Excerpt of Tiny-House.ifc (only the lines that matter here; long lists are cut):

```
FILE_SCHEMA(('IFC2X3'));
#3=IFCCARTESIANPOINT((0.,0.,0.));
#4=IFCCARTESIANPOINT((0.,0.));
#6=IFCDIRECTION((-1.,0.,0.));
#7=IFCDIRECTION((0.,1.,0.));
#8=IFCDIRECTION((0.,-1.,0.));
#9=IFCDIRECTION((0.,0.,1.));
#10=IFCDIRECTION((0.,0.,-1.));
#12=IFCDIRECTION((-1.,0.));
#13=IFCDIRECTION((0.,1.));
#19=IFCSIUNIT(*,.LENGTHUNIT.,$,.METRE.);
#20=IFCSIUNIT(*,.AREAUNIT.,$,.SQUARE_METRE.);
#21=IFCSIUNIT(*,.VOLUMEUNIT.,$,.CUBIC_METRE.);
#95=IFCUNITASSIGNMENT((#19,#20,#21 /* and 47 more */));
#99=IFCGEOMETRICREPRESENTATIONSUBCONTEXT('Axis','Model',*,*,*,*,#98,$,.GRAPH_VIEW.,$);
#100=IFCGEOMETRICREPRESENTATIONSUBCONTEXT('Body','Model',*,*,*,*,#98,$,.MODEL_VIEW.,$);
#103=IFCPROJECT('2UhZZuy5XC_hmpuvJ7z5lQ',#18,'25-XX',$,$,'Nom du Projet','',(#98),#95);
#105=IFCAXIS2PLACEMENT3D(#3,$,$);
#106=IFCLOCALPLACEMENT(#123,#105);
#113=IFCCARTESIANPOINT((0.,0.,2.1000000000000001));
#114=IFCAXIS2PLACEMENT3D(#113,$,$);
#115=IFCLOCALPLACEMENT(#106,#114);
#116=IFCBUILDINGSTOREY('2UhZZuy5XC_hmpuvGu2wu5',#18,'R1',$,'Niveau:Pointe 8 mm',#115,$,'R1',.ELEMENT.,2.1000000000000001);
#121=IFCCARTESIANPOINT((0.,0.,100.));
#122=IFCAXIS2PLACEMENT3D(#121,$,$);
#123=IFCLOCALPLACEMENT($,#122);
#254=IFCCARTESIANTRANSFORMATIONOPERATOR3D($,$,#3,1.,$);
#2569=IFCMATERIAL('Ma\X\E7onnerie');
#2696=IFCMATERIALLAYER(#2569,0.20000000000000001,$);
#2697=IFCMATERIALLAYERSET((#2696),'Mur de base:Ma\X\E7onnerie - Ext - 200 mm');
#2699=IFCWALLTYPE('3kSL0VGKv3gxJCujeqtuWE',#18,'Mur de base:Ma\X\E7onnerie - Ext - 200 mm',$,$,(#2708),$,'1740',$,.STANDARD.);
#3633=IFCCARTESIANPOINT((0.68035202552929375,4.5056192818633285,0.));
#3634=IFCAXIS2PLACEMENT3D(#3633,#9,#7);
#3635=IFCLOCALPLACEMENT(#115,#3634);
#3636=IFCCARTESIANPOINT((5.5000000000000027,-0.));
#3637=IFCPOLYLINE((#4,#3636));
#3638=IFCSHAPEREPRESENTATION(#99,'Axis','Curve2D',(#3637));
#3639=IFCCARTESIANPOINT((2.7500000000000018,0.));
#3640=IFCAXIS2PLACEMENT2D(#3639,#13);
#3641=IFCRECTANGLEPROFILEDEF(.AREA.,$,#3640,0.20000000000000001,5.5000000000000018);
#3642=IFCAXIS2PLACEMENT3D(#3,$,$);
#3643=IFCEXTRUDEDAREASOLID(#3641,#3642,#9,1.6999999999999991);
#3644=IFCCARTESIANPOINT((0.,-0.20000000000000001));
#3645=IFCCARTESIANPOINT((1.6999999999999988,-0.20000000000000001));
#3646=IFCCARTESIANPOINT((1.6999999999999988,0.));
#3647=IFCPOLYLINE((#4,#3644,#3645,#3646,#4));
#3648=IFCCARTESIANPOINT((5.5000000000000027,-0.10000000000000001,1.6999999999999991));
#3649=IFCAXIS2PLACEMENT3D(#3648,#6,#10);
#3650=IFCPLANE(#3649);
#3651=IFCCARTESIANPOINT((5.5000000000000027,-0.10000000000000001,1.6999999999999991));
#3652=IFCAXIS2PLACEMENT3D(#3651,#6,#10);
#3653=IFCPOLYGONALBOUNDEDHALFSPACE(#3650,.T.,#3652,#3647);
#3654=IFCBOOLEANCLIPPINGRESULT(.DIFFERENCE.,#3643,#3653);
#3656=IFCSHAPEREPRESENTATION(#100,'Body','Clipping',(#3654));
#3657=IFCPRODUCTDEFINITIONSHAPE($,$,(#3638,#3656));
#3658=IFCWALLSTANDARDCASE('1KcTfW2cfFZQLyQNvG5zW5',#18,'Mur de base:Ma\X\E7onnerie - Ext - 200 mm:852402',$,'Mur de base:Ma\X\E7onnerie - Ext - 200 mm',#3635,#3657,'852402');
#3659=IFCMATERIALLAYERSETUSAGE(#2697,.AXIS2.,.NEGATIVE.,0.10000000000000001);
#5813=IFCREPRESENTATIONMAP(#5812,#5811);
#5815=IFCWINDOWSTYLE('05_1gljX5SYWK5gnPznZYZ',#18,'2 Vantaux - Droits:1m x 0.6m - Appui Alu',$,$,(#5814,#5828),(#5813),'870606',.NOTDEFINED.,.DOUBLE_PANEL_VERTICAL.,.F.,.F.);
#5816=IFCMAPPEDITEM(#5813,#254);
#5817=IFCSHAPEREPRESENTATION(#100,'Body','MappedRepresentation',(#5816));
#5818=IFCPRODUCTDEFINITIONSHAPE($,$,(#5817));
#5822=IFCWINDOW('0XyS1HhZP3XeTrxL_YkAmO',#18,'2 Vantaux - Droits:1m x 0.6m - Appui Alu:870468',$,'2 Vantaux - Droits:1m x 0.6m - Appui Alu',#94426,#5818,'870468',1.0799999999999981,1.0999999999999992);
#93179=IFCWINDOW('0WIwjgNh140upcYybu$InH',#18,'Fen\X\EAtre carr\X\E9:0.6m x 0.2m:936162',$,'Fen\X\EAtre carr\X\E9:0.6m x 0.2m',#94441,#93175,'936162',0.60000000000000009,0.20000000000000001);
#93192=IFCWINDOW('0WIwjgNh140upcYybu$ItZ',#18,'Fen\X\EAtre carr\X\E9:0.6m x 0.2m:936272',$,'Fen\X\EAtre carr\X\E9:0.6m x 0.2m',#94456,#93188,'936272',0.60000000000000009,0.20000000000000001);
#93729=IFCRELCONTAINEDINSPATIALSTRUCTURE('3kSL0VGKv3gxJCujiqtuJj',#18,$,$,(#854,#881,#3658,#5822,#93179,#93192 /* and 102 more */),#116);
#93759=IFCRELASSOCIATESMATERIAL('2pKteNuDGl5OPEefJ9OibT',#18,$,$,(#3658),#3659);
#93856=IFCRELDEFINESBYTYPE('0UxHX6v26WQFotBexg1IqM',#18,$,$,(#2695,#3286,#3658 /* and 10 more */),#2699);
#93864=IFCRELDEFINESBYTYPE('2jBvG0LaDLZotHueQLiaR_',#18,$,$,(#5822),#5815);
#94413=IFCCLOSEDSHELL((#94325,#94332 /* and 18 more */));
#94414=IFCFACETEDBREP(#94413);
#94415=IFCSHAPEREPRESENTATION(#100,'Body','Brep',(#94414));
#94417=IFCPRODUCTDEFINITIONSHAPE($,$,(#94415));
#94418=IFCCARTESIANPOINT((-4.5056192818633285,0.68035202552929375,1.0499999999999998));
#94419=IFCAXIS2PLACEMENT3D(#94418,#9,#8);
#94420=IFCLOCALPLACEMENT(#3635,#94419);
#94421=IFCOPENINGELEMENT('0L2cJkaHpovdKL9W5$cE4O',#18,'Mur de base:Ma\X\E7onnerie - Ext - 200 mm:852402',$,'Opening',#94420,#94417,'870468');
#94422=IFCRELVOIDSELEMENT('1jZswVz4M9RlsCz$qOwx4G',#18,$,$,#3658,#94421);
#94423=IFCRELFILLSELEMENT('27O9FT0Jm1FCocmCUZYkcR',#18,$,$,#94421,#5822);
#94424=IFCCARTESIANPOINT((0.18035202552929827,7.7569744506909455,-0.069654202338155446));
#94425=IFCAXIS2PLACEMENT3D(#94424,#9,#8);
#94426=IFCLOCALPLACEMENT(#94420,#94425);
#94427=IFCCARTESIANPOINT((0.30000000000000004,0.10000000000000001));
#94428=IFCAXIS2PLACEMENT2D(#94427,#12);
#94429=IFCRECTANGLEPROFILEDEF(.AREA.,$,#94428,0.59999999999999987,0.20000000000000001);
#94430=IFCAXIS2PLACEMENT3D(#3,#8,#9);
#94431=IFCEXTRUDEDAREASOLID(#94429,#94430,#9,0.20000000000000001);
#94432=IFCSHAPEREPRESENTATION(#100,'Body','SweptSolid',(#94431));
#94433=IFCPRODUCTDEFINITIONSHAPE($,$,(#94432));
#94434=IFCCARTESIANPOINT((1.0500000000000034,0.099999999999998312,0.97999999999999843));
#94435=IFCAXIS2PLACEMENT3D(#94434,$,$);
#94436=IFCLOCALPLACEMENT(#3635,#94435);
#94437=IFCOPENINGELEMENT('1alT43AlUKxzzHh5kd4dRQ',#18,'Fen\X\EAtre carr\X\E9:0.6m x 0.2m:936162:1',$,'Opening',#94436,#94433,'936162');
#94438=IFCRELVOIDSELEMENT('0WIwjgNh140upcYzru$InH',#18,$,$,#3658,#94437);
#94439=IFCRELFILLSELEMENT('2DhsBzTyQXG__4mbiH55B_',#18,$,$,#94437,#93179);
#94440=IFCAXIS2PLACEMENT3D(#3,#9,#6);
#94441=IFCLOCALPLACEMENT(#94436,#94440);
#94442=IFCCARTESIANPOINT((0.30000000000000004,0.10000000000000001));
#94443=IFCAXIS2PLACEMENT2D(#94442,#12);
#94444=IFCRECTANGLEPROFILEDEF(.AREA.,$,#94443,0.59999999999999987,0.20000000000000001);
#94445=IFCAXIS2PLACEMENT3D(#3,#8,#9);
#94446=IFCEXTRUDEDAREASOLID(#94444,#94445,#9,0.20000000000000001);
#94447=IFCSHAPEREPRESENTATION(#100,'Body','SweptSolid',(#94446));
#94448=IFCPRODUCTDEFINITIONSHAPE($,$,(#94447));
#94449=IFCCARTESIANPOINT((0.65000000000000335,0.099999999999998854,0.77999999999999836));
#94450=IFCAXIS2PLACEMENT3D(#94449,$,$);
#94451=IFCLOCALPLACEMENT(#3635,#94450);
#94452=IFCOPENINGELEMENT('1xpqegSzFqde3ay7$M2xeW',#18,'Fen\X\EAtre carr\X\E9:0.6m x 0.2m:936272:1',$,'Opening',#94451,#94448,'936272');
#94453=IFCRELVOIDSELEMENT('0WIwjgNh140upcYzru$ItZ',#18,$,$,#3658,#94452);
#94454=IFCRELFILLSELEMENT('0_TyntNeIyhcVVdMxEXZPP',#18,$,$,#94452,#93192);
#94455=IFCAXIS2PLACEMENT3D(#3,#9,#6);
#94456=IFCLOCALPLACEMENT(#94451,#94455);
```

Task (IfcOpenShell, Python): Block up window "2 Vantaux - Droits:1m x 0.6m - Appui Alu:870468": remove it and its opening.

```python
import ifcopenshell
import ifcopenshell.api.feature
import ifcopenshell.api.root
import ifcopenshell.geom
import ifcopenshell.util.shape

model = ifcopenshell.open("Tiny-House.ifc")
settings = ifcopenshell.geom.settings()


def volume(element):
    """Net volume in cubic metres, openings subtracted."""
    shape = ifcopenshell.geom.create_shape(settings, element)
    return ifcopenshell.util.shape.get_volume(shape.geometry)


window = model.by_guid("0XyS1HhZP3XeTrxL_YkAmO")
opening = window.FillsVoids[0].RelatingOpeningElement
wall = opening.VoidsElements[0].RelatingBuildingElement
before = volume(wall)

ifcopenshell.api.root.remove_product(model, product=window)
ifcopenshell.api.feature.remove_feature(model, feature=opening)

after = volume(wall)

print(f"wall volume {before:.3f} -> {after:.3f} m3")

model.write("Tiny-House_rev.ifc")
```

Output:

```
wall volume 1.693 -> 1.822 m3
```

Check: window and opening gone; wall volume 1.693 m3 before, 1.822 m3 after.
